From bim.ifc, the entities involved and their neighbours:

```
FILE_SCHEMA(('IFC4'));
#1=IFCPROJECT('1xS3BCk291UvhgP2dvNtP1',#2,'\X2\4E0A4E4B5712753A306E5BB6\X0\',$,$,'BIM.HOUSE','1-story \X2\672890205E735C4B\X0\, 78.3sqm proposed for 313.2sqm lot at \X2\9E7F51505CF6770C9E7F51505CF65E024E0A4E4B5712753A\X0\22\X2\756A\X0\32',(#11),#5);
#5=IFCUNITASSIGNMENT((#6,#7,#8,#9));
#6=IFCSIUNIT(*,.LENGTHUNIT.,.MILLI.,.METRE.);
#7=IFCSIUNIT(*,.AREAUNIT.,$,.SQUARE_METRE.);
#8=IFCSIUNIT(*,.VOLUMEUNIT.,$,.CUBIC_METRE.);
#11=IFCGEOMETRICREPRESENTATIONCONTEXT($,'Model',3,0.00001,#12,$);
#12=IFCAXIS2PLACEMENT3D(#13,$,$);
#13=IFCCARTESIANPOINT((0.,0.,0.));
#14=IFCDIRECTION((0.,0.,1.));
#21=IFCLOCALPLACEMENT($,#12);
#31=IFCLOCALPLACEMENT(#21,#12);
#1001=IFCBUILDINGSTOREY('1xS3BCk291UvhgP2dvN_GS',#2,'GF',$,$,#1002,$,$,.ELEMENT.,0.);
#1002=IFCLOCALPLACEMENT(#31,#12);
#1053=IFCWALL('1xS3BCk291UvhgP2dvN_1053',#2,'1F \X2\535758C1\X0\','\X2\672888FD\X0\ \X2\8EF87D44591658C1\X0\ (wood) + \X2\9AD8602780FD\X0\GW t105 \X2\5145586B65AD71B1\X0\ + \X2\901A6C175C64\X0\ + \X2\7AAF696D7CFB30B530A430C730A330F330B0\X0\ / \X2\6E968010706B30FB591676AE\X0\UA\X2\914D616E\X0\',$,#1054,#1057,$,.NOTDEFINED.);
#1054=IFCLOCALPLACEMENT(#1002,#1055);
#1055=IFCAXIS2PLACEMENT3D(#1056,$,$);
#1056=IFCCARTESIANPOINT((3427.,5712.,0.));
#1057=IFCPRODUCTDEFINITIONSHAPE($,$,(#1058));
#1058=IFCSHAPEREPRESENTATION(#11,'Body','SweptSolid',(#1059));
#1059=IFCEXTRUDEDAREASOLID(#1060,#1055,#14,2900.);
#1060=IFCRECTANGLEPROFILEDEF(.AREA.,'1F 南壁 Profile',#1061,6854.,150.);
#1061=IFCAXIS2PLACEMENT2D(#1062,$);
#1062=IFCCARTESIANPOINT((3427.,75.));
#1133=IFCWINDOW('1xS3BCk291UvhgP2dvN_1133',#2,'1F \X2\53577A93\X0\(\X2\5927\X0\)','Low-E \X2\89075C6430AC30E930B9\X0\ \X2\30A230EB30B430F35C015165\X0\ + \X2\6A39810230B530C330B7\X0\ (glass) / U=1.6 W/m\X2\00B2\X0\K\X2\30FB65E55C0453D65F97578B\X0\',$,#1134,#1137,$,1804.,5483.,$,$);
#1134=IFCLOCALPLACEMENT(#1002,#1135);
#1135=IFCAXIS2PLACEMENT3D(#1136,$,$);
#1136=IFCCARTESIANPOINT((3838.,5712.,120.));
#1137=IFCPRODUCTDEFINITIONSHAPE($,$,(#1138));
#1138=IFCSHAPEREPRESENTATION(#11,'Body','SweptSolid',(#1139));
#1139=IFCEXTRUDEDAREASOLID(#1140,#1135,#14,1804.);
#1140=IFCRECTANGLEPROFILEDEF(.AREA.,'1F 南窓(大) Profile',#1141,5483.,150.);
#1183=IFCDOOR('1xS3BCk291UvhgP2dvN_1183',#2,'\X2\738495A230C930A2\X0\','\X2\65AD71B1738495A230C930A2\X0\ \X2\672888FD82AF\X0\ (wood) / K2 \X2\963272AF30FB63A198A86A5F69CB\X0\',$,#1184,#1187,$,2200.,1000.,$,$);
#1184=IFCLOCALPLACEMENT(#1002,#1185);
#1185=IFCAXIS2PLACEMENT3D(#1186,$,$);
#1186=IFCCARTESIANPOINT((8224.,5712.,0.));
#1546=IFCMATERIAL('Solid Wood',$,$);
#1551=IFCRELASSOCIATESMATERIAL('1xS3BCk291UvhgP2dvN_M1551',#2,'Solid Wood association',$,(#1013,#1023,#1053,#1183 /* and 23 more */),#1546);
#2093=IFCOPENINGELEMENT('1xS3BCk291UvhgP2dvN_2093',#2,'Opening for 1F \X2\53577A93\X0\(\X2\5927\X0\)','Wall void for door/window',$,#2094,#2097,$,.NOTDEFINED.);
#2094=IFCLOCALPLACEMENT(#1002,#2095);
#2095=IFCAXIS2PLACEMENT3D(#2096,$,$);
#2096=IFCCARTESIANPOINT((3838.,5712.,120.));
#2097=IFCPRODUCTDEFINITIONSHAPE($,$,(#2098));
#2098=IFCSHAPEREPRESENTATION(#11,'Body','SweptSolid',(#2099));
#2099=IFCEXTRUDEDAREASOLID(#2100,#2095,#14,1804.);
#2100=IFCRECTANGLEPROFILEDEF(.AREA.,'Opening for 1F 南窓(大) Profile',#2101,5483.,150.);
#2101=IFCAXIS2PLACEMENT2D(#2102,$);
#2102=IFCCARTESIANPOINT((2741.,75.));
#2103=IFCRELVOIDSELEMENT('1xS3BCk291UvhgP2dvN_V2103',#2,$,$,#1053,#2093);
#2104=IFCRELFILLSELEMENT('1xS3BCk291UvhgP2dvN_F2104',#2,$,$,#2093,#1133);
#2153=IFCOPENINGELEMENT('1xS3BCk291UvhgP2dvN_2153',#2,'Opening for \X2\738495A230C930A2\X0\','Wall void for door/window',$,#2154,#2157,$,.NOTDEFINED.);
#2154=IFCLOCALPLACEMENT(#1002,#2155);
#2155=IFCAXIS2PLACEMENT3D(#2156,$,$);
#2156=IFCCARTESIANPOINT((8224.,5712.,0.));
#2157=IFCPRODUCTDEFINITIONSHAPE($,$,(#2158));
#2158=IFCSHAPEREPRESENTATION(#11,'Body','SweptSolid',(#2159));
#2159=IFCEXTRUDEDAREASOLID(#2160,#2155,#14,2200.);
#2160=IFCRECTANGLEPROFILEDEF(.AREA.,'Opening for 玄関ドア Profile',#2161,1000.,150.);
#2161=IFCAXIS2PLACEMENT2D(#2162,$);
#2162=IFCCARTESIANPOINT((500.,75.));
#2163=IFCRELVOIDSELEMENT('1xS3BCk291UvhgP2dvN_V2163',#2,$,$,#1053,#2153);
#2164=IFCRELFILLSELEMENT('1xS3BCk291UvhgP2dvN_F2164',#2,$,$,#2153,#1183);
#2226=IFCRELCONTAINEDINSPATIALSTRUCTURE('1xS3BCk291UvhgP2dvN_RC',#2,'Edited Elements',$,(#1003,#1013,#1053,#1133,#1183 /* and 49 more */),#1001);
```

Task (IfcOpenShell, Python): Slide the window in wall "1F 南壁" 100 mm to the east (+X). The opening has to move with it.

```python
import ifcopenshell
import ifcopenshell.api.geometry
import ifcopenshell.util.placement

model = ifcopenshell.open("bim.ifc")

window = model.by_id(1133)
opening = window.FillsVoids[0].RelatingOpeningElement
wall = opening.VoidsElements[0].RelatingBuildingElement

wall_matrix = ifcopenshell.util.placement.get_local_placement(wall.ObjectPlacement)
shift = wall_matrix[:3, 0] * 100.0
before = ifcopenshell.util.placement.get_local_placement(window.ObjectPlacement)[:3, 3].copy()

# The window is not placed relative to its opening, so move both.
for product in (opening, window):
    matrix = ifcopenshell.util.placement.get_local_placement(product.ObjectPlacement)
    matrix[:3, 3] += shift
    ifcopenshell.api.geometry.edit_object_placement(model, product=product, matrix=matrix, is_si=False)

after = ifcopenshell.util.placement.get_local_placement(window.ObjectPlacement)[:3, 3]
print("window moved by", (after - before).round(3) + 0.0)

model.write("bim_rev.ifc")
```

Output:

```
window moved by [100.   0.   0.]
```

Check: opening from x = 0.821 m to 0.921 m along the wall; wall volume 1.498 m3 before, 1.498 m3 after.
